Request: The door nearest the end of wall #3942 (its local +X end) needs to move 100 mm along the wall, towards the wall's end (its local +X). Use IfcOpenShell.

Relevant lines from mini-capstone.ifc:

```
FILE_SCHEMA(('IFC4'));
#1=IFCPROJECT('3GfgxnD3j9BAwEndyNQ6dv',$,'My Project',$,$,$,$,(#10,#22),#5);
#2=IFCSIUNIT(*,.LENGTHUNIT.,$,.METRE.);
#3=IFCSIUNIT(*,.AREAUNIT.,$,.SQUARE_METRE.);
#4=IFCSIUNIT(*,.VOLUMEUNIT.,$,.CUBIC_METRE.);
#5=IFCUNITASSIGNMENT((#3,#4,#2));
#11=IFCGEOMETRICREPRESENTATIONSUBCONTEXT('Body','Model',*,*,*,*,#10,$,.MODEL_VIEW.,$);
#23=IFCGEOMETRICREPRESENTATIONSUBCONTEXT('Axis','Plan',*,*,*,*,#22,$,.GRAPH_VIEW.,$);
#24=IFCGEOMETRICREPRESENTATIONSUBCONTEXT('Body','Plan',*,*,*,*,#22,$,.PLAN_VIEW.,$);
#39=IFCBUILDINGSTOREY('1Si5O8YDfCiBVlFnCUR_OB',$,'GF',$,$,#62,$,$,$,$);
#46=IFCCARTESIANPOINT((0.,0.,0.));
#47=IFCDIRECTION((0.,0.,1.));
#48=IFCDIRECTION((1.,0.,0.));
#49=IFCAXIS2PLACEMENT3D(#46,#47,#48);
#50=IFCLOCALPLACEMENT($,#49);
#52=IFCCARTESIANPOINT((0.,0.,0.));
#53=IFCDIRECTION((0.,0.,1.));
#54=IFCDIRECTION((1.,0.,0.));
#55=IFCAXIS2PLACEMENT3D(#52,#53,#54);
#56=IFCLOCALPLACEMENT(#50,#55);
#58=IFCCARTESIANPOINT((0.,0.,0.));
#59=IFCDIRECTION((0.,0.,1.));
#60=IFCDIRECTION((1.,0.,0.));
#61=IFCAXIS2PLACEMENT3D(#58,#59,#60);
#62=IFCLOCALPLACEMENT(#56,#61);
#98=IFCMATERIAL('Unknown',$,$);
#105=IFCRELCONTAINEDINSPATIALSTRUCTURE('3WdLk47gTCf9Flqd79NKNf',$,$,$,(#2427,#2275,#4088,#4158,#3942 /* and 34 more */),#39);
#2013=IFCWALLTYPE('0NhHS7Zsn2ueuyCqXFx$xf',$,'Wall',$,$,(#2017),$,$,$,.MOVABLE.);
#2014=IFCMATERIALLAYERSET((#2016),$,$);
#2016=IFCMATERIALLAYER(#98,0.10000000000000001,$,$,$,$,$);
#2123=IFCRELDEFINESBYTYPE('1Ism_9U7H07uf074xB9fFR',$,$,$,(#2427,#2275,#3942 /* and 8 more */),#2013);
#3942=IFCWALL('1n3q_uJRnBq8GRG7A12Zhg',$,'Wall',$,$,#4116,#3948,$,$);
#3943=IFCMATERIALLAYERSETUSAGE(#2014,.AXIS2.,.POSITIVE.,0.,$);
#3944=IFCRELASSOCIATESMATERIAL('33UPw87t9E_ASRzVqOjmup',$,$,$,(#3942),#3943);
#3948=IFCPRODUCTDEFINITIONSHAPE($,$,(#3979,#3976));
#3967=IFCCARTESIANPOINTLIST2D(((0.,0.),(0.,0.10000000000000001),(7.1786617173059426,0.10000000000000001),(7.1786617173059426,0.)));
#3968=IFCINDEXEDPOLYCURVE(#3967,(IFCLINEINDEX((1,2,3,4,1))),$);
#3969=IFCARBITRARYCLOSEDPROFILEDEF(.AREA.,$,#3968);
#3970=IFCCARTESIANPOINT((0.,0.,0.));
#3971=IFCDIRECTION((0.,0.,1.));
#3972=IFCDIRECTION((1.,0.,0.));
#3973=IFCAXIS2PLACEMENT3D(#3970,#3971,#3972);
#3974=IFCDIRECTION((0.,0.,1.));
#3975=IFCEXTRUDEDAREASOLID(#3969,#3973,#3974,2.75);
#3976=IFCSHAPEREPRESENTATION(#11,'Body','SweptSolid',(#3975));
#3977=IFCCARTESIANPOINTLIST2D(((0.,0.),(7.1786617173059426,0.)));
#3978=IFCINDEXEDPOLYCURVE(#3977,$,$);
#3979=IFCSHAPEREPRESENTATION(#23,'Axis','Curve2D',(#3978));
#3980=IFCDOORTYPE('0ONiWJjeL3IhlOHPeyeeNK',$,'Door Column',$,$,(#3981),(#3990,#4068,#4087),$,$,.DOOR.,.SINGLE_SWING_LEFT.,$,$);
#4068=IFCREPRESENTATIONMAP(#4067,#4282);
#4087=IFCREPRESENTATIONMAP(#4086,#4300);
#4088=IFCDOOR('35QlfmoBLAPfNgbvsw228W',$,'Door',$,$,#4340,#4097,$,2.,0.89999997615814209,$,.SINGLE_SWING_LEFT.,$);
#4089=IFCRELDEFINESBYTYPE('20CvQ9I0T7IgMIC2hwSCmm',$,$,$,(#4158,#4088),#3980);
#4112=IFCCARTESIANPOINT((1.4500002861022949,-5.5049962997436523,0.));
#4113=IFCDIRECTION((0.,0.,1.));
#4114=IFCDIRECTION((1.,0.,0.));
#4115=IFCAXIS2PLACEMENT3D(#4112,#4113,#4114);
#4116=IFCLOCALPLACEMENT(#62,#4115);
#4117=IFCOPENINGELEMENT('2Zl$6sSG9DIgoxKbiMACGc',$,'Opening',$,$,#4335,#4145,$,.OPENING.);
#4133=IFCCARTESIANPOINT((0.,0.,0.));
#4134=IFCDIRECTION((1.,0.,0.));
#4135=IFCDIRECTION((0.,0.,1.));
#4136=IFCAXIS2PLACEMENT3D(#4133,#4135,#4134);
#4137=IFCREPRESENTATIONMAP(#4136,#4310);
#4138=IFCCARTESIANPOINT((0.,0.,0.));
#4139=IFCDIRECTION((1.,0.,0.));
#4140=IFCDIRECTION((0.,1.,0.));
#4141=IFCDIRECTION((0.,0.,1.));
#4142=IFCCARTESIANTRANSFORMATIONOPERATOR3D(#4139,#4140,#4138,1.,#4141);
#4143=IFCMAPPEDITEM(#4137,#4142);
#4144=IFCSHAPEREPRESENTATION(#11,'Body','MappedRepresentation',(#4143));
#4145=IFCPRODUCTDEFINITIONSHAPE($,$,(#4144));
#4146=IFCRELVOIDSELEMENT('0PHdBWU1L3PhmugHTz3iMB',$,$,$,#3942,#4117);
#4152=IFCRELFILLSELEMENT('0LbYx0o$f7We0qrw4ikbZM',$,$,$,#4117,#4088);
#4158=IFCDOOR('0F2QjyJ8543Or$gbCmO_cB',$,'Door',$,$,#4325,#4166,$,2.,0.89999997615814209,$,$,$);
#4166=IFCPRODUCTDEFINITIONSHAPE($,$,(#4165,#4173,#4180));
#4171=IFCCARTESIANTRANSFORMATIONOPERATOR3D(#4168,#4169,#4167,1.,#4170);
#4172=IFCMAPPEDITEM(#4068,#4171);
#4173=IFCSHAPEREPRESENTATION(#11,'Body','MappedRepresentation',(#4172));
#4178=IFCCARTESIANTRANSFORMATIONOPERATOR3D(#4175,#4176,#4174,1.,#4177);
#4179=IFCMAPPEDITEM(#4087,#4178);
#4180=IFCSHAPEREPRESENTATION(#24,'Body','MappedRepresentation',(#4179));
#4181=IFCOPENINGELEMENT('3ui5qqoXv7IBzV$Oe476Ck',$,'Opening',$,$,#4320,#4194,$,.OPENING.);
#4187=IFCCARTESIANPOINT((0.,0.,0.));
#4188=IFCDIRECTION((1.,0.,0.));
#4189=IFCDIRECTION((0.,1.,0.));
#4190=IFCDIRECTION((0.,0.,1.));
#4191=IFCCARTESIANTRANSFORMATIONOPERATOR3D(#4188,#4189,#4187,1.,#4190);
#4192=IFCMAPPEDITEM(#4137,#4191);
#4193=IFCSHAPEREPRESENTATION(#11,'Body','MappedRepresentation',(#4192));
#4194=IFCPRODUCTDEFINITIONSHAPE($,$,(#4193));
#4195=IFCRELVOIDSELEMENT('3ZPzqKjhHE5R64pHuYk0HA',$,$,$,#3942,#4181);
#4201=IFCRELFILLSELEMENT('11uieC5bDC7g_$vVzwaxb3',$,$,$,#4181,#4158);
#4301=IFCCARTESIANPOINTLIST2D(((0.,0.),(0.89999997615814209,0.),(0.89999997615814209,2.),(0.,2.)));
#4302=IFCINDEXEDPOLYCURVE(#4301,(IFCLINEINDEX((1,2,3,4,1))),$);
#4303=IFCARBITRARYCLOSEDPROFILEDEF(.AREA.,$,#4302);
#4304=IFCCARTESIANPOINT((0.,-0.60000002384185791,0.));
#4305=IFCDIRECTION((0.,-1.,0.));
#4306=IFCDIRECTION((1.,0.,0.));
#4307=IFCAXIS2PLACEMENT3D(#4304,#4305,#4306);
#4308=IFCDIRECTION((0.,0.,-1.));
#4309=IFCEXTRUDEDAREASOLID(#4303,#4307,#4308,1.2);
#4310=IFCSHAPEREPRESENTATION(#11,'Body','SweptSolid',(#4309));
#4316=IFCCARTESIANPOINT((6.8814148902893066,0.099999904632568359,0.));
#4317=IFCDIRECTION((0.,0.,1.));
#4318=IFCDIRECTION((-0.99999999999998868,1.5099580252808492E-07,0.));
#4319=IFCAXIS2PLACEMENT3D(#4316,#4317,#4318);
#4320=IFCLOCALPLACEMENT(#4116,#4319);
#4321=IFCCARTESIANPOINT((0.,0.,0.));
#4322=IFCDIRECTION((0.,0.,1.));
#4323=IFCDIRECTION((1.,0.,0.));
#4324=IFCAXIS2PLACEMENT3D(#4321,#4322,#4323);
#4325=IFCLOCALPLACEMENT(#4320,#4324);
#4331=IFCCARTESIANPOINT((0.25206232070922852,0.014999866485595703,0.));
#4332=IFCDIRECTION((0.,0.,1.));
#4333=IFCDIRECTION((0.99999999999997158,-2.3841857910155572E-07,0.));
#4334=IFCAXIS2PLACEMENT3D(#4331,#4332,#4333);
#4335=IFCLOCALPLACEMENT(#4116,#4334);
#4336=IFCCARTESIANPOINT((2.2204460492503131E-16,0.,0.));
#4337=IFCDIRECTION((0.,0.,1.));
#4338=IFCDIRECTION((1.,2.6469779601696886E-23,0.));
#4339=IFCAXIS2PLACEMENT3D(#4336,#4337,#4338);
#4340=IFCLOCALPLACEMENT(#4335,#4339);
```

```python
import ifcopenshell
import ifcopenshell.api.geometry
import ifcopenshell.util.placement

model = ifcopenshell.open("mini-capstone.ifc")

door = model.by_guid("0F2QjyJ8543Or$gbCmO_cB")
opening = door.FillsVoids[0].RelatingOpeningElement
wall = opening.VoidsElements[0].RelatingBuildingElement

wall_matrix = ifcopenshell.util.placement.get_local_placement(wall.ObjectPlacement)
shift = wall_matrix[:3, 0] * 0.1
before = ifcopenshell.util.placement.get_local_placement(door.ObjectPlacement)[:3, 3].copy()

# The door is placed relative to its opening, so it follows when the opening moves.
matrix = ifcopenshell.util.placement.get_local_placement(opening.ObjectPlacement)
matrix[:3, 3] += shift
ifcopenshell.api.geometry.edit_object_placement(
    model, product=opening, matrix=matrix, is_si=False, should_transform_children=True
)

after = ifcopenshell.util.placement.get_local_placement(door.ObjectPlacement)[:3, 3]
print("door moved by", (after - before).round(3) + 0.0)

model.write("mini-capstone_v2.ifc")
```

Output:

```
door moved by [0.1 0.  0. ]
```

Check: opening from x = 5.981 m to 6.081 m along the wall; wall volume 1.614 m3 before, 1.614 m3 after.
